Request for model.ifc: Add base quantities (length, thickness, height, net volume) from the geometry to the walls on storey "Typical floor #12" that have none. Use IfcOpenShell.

First a look at what the model holds.

```python
import ifcopenshell
import ifcopenshell.util.element
import ifcopenshell.util.unit

model = ifcopenshell.open("model.ifc")
print(model.schema)
for unit_type in ("LENGTHUNIT", "AREAUNIT", "VOLUMEUNIT"):
    print(unit_type, ifcopenshell.util.unit.calculate_unit_scale(model, unit_type))
storey = next(s for s in model.by_type("IfcBuildingStorey") if s.Name == "Typical floor #12")
walls = [e for e in ifcopenshell.util.element.get_decomposition(storey) if e.is_a("IfcWall")]
for e in sorted(walls, key=lambda e: e.id()):
    print(e.id(), e.is_a(), e.Name, list(ifcopenshell.util.element.get_psets(e, qtos_only=True)), sep=" | ")
```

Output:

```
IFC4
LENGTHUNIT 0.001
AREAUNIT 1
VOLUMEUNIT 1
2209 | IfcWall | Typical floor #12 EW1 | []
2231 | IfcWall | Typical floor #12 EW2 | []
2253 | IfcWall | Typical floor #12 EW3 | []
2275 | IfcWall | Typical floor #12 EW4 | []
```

```python
import ifcopenshell
import ifcopenshell.api.pset
import ifcopenshell.geom
import ifcopenshell.util.element
import ifcopenshell.util.shape
import ifcopenshell.util.unit

model = ifcopenshell.open("model.ifc")
unit_scale = ifcopenshell.util.unit.calculate_unit_scale(model)
volume_scale = ifcopenshell.util.unit.calculate_unit_scale(model, "VOLUMEUNIT")
settings = ifcopenshell.geom.settings()

storey = next(s for s in model.by_type("IfcBuildingStorey") if s.Name == "Typical floor #12")
walls = [e for e in ifcopenshell.util.element.get_decomposition(storey) if e.is_a("IfcWall")]

for e in sorted(walls, key=lambda e: e.id()):
    if ifcopenshell.util.element.get_psets(e, qtos_only=True, should_inherit=False):
        continue
    # Geometry comes back in metres, in the element's own axes.
    shape = ifcopenshell.geom.create_shape(settings, e)
    values = {
        "Length": ifcopenshell.util.shape.get_x(shape.geometry) / unit_scale,
        "Width": ifcopenshell.util.shape.get_y(shape.geometry) / unit_scale,
        "Height": ifcopenshell.util.shape.get_z(shape.geometry) / unit_scale,
        "NetVolume": ifcopenshell.util.shape.get_volume(shape.geometry) / volume_scale,
    }
    qto = ifcopenshell.api.pset.add_qto(model, product=e, name="Qto_WallBaseQuantities")
    ifcopenshell.api.pset.edit_qto(model, qto=qto, properties=values)
    print(e.id(), {k: round(v, 3) for k, v in values.items()})

model.write("model_v2.ifc")
```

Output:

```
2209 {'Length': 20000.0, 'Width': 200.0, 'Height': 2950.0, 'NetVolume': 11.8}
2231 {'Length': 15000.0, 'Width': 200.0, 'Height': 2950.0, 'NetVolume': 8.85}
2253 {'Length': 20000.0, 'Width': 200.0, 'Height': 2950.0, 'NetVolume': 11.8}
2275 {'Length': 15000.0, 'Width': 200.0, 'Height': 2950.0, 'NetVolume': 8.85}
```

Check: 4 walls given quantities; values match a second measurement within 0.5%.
